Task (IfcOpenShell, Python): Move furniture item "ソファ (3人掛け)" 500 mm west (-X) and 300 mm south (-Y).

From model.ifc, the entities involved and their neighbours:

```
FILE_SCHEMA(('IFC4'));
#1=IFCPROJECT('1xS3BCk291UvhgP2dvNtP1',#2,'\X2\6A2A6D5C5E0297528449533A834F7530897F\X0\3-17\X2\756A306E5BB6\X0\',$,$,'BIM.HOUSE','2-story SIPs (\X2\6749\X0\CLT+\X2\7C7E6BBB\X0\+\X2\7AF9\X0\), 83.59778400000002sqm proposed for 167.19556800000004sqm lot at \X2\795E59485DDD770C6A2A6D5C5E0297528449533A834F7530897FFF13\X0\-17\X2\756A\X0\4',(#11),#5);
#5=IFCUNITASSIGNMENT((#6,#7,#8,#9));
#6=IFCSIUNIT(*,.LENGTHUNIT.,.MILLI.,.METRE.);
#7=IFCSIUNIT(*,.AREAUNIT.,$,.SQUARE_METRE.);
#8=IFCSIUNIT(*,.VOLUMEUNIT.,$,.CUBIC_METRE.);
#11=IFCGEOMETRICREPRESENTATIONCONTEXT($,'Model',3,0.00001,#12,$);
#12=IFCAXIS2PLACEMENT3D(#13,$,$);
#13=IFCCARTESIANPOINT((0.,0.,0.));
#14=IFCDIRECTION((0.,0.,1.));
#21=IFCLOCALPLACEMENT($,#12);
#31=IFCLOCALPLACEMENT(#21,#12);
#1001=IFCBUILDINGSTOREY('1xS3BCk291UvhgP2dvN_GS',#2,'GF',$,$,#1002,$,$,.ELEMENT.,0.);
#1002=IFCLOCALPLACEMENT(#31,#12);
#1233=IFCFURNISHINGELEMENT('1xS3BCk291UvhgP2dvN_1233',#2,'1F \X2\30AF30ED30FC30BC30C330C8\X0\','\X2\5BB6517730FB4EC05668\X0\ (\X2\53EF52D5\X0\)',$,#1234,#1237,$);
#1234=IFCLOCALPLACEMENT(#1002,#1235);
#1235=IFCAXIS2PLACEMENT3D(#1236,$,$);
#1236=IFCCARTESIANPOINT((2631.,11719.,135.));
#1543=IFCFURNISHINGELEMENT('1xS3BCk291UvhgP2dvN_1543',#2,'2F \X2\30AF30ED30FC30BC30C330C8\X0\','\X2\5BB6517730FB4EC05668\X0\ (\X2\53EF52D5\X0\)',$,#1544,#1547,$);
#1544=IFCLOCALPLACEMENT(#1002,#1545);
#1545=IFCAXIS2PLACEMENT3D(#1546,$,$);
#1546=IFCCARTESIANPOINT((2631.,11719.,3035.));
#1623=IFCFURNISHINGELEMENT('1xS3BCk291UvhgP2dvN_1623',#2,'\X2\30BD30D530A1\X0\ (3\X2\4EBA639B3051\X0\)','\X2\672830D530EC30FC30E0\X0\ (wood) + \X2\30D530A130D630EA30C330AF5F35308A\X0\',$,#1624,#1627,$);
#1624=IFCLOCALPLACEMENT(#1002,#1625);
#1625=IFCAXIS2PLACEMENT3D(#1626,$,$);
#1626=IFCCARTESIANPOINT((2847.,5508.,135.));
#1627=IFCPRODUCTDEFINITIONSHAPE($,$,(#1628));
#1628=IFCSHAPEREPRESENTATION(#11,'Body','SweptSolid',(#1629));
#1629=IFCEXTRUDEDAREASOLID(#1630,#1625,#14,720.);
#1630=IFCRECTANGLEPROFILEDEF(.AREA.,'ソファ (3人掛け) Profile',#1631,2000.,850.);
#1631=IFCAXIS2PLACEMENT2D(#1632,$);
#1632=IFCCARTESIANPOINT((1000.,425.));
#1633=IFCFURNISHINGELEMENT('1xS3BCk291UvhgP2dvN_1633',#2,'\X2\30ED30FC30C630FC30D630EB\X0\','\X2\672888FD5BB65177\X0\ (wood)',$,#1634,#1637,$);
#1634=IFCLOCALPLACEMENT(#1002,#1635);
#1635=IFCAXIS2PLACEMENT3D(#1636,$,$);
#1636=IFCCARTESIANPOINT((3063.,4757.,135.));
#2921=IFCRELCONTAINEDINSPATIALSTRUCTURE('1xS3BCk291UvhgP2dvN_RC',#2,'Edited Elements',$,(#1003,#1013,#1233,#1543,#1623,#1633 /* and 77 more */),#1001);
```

```python
import ifcopenshell
import ifcopenshell.api.geometry
import ifcopenshell.util.placement
import ifcopenshell.util.unit

model = ifcopenshell.open("model.ifc")
unit_scale = ifcopenshell.util.unit.calculate_unit_scale(model)

item = model.by_id(1623)
matrix = ifcopenshell.util.placement.get_local_placement(item.ObjectPlacement)
matrix[0, 3] -= 0.5 / unit_scale
matrix[1, 3] -= 0.3 / unit_scale
ifcopenshell.api.geometry.edit_object_placement(model, product=item, matrix=matrix, is_si=False)

print(ifcopenshell.util.placement.get_local_placement(item.ObjectPlacement).round(3) + 0.0)

model.write("model_v2.ifc")
```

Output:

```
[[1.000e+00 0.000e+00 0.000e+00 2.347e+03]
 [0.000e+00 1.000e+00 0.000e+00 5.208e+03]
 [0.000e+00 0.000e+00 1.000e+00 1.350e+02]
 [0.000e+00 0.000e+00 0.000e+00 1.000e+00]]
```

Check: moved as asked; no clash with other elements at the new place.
